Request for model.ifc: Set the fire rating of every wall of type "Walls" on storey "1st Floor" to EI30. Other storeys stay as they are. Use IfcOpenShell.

First a look at what the model holds.

```python
import ifcopenshell
import ifcopenshell.util.element

model = ifcopenshell.open("model.ifc")
print(model.schema)
storey = next(s for s in model.by_type("IfcBuildingStorey") if s.Name == "1st Floor")
walls = [e for e in ifcopenshell.util.element.get_decomposition(storey) if e.is_a("IfcWall")]
seen = {}
for e in walls:
    element_type = ifcopenshell.util.element.get_type(e)
    key = (element_type.Name if element_type != e and element_type else None, ifcopenshell.util.element.get_pset(e, "Pset_WallCommon", "FireRating"))
    seen[key] = seen.get(key, 0) + 1
for (name, value), count in sorted(seen.items(), key=str):
    print(count, "x", name, "|", value)
```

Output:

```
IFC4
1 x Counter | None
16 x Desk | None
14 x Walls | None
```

```python
import ifcopenshell
import ifcopenshell.api.pset
import ifcopenshell.util.element

model = ifcopenshell.open("model.ifc")

storey = next(s for s in model.by_type("IfcBuildingStorey") if s.Name == "1st Floor")
walls = [e for e in ifcopenshell.util.element.get_decomposition(storey) if e.is_a("IfcWall")]

count = 0
for e in walls:
    element_type = ifcopenshell.util.element.get_type(e)
    if element_type in (None, e) or element_type.Name != "Walls":
        continue
    # add_pset returns the element's existing set when there is one.
    pset = ifcopenshell.api.pset.add_pset(model, product=e, name="Pset_WallCommon")
    ifcopenshell.api.pset.edit_pset(model, pset=pset, properties={"FireRating": "EI30"})
    count += 1

print(count, "walls updated")

model.write("model-out.ifc")
```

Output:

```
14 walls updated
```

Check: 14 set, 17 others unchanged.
